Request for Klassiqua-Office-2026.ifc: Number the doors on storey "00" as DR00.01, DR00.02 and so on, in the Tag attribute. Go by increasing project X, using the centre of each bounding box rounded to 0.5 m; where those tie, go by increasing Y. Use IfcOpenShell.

First a look at what the model holds.

```python
import ifcopenshell
import ifcopenshell.util.element
import ifcopenshell.util.placement

model = ifcopenshell.open("Klassiqua-Office-2026.ifc")
print(model.schema)
storey = next(s for s in model.by_type("IfcBuildingStorey") if s.Name == "00")
doors = [e for e in ifcopenshell.util.element.get_decomposition(storey) if e.is_a("IfcDoor")]
for e in sorted(doors, key=lambda e: e.id()):
    origin = ifcopenshell.util.placement.get_local_placement(e.ObjectPlacement)[:3, 3]
    print(e.id(), e.Tag, e.Name, origin.round(2) + 0.0, sep=" | ")
```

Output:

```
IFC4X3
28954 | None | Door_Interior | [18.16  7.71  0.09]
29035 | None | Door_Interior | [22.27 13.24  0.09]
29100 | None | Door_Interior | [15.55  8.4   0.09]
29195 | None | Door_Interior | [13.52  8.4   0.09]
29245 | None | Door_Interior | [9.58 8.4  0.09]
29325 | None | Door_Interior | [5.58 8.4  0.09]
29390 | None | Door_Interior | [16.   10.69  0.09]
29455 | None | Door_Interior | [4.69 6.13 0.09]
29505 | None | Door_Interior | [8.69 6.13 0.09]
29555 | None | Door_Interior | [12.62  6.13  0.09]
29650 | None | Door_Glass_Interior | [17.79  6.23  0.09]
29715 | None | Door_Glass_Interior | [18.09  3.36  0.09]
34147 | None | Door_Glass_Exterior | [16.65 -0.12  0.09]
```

```python
import ifcopenshell
import ifcopenshell.geom
import ifcopenshell.util.element
import ifcopenshell.util.shape

model = ifcopenshell.open("Klassiqua-Office-2026.ifc")
settings = ifcopenshell.geom.settings()
settings.set("use-world-coords", True)


def centre(element):
    shape = ifcopenshell.geom.create_shape(settings, element)
    return ifcopenshell.util.shape.get_bbox_centroid(shape.geometry)


storey = next(s for s in model.by_type("IfcBuildingStorey") if s.Name == "00")
doors = [e for e in ifcopenshell.util.element.get_decomposition(storey) if e.is_a("IfcDoor")]

# Insertion points can sit at a corner or the storey origin, so sort by the geometry (in metres).
centres = {e: centre(e) for e in doors}
doors.sort(key=lambda e: (round(centres[e][0] / 0.5), centres[e][1]))

for i, e in enumerate(doors, start=1):
    number = f"DR00.{i:02d}"
    e.Tag = number
    print(e.id(), number)

model.write("Klassiqua-Office-2026-out.ifc")
```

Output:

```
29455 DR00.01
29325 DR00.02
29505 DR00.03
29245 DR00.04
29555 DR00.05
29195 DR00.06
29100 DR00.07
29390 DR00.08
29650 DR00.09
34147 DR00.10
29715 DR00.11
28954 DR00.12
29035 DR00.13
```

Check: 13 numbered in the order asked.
